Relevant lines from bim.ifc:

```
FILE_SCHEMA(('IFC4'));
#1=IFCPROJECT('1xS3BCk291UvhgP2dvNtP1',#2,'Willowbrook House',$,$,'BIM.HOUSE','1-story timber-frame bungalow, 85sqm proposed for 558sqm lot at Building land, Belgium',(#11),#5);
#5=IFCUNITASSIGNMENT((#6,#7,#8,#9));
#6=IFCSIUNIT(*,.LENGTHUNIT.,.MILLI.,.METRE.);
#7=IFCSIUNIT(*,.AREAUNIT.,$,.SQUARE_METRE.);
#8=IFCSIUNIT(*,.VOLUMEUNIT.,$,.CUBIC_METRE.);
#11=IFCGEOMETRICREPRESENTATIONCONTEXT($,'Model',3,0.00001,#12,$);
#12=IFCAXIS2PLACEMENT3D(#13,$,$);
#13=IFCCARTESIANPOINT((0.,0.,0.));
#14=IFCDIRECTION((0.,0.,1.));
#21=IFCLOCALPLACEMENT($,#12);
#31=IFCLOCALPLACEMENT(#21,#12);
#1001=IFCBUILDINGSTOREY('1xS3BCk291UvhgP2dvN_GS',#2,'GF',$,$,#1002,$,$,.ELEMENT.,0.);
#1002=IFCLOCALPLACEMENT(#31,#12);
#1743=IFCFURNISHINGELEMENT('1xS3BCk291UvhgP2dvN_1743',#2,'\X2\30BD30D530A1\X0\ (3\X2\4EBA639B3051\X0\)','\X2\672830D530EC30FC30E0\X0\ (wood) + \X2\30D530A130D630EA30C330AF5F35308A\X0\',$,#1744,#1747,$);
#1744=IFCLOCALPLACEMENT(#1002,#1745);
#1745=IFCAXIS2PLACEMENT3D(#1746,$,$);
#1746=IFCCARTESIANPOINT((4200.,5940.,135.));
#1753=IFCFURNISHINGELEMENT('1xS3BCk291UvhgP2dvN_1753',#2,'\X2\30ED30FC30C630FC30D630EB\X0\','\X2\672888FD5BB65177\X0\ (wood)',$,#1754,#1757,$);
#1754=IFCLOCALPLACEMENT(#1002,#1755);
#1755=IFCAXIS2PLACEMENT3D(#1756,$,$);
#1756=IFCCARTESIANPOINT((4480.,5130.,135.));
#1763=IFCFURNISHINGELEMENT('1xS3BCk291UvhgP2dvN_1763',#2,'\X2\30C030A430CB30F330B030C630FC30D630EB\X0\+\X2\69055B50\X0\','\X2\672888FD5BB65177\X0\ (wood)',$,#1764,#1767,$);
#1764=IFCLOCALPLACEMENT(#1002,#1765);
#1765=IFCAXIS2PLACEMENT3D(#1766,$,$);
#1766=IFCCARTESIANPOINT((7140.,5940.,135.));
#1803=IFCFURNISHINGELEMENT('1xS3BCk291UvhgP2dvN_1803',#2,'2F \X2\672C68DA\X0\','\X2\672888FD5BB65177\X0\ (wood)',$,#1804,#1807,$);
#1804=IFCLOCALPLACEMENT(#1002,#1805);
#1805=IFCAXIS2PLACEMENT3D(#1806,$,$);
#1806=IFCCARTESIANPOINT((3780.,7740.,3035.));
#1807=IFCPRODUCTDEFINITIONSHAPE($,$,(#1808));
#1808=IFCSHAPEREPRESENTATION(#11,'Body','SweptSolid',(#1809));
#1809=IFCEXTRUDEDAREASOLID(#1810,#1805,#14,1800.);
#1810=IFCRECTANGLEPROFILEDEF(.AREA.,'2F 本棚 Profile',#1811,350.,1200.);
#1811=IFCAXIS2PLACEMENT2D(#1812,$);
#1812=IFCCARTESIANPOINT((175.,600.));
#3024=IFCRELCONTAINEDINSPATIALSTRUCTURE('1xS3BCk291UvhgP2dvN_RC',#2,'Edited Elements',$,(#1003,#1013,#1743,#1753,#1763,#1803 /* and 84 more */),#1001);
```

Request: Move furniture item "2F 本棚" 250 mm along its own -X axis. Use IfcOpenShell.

```python
import ifcopenshell
import ifcopenshell.api.geometry
import ifcopenshell.util.placement
import ifcopenshell.util.unit

model = ifcopenshell.open("bim.ifc")
unit_scale = ifcopenshell.util.unit.calculate_unit_scale(model)

item = model.by_guid("1xS3BCk291UvhgP2dvN_1803")
matrix = ifcopenshell.util.placement.get_local_placement(item.ObjectPlacement)
matrix[:3, 3] -= matrix[:3, 0] * 0.25 / unit_scale
ifcopenshell.api.geometry.edit_object_placement(model, product=item, matrix=matrix, is_si=False)

print(ifcopenshell.util.placement.get_local_placement(item.ObjectPlacement).round(3) + 0.0)

model.write("bim-out.ifc")
```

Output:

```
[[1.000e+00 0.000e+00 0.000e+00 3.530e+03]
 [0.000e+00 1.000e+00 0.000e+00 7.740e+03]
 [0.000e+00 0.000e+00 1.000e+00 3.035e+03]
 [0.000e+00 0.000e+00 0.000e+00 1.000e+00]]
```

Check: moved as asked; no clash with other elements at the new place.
